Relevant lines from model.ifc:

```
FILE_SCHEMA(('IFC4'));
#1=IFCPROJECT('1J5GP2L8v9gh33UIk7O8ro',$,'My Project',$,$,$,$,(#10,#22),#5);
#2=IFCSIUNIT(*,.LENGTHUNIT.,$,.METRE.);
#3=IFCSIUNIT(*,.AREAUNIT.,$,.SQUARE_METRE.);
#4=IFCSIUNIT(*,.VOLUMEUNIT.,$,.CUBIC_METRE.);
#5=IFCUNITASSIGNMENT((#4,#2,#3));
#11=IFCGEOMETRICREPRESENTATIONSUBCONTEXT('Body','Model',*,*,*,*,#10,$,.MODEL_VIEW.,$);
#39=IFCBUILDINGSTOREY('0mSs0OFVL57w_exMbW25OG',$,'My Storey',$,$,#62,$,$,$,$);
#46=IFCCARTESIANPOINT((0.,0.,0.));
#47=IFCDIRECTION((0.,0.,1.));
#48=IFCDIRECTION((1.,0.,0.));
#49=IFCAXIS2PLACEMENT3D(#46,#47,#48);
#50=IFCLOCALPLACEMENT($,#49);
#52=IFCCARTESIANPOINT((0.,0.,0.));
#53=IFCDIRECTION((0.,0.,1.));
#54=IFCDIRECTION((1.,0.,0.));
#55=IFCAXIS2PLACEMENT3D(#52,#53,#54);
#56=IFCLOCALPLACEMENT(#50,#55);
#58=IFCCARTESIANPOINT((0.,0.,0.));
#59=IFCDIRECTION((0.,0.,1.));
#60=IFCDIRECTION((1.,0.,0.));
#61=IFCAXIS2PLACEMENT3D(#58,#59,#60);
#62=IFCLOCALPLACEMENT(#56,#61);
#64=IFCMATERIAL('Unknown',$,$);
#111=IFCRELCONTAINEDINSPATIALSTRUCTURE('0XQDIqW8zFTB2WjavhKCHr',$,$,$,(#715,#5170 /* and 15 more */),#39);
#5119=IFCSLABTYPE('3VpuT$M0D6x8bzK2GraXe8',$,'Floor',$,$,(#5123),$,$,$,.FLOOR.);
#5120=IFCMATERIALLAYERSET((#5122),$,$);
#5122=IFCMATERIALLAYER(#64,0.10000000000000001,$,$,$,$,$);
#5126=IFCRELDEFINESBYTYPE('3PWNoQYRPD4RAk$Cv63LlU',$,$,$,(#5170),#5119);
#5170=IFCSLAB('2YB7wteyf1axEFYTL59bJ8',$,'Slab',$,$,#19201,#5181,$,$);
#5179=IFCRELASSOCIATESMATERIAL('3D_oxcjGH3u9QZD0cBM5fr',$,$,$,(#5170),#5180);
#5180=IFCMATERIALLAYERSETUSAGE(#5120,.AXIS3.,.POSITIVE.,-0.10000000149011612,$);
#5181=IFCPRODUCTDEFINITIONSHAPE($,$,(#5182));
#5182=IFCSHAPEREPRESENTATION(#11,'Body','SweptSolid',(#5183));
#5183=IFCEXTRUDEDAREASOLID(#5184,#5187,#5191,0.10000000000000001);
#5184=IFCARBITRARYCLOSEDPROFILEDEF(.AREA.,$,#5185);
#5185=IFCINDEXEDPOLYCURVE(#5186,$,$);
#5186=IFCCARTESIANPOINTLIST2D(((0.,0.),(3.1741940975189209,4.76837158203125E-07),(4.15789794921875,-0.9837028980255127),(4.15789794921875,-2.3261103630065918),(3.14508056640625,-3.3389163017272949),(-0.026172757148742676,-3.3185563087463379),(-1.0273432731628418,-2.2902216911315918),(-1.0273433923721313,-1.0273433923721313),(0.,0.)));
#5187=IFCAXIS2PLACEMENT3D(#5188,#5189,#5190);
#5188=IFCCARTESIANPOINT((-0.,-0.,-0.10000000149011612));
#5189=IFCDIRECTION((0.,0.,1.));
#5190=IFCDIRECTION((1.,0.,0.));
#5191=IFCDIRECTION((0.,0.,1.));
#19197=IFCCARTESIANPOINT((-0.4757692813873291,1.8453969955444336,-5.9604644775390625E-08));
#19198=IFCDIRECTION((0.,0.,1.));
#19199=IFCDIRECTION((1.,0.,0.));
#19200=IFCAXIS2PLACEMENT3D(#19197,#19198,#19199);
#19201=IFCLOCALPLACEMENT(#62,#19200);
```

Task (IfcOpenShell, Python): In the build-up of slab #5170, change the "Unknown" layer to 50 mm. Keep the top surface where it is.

```python
import ifcopenshell
import ifcopenshell.util.element
import ifcopenshell.util.representation
import ifcopenshell.util.unit

model = ifcopenshell.open("model.ifc")
unit_scale = ifcopenshell.util.unit.calculate_unit_scale(model)

layer_set = model.by_id(5120)
layer = next(l for l in layer_set.MaterialLayers if l.Material and l.Material.Name == "Unknown")
change = 0.05 / unit_scale - layer.LayerThickness
layer.LayerThickness += change

# Geometry does not follow the layer set by itself.
slabs = [e for e in ifcopenshell.util.element.get_elements_by_material(model, layer_set) if e.is_a("IfcSlab")]
for slab in sorted(slabs, key=lambda e: e.id()):
    body = ifcopenshell.util.representation.get_representation(slab, "Model", "Body")
    solid = body.Items[0]
    old_depth = solid.Depth
    solid.Depth += change
    # Extruded upwards: lower the start of the extrusion so the top stays.
    x, y, z = solid.Position.Location.Coordinates
    solid.Position.Location = model.createIfcCartesianPoint((x, y, z - change))
    print(slab.id(), f"{old_depth:g} -> {solid.Depth:g}")

# The layers are counted up from the underside, which has moved.
for usage in {ifcopenshell.util.element.get_material(slab) for slab in slabs}:
    usage.OffsetFromReferenceLine -= change

model.write("model_rev.ifc")
```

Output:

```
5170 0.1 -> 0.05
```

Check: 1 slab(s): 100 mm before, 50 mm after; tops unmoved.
